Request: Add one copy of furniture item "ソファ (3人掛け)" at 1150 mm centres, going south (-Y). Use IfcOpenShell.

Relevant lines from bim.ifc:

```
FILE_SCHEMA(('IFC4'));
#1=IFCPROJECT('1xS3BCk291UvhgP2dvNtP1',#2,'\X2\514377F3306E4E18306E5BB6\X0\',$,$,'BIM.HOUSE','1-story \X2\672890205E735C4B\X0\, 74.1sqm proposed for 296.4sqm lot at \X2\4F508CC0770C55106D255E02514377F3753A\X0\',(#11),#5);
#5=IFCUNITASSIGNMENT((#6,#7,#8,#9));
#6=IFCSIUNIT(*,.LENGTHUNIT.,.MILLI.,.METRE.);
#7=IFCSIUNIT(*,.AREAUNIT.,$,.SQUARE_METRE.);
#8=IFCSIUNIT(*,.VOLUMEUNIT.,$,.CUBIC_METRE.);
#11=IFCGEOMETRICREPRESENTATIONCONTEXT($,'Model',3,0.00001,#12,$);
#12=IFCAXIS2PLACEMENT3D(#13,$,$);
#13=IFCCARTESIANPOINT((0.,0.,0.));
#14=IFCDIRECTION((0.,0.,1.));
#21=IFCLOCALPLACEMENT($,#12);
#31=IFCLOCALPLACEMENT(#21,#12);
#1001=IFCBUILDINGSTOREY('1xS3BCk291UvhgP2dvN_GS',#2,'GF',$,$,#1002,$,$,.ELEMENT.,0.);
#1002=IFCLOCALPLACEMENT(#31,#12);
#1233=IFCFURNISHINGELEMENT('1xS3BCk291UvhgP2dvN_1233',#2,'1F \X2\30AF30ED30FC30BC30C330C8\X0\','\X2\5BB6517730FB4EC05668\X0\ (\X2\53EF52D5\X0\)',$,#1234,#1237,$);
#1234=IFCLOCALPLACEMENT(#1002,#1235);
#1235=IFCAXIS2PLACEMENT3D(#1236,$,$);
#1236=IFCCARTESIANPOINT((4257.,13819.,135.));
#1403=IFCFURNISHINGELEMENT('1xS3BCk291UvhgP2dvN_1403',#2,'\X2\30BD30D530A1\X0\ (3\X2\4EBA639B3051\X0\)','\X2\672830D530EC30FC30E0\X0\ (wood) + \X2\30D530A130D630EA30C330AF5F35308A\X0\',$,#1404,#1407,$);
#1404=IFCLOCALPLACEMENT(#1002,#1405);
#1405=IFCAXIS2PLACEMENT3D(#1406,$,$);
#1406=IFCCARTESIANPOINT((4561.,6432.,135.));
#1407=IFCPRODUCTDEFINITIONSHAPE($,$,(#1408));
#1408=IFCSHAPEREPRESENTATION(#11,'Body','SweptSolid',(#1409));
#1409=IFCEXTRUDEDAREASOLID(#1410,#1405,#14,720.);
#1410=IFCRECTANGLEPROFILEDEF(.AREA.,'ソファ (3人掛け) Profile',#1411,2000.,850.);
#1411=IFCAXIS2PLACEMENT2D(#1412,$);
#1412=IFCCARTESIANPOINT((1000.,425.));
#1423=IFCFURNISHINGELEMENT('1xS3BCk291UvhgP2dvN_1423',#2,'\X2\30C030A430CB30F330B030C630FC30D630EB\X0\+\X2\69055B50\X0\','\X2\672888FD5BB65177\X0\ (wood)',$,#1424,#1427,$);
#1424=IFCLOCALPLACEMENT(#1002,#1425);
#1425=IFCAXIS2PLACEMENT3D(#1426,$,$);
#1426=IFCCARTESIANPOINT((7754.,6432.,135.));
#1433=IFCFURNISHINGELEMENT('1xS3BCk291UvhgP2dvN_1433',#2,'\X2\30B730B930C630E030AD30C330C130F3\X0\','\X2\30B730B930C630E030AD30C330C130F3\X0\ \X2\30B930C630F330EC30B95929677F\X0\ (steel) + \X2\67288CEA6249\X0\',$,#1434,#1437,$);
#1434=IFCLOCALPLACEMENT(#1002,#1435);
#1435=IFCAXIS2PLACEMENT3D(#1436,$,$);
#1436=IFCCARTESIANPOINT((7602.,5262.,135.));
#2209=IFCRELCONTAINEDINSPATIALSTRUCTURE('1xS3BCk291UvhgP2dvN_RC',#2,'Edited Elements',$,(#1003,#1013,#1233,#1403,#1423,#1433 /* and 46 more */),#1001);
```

```python
import numpy as np
import ifcopenshell
import ifcopenshell.api.geometry
import ifcopenshell.api.root
import ifcopenshell.util.element
import ifcopenshell.util.placement

model = ifcopenshell.open("bim.ifc")


def reuse_history(source, copy):
    """copy_class also copies each property set's owner history, people and application; keep the originals."""
    for rel in copy.IsDefinedBy:
        if rel.is_a("IfcRelDefinesByProperties") and (history := rel.RelatingPropertyDefinition.OwnerHistory):
            rel.RelatingPropertyDefinition.OwnerHistory = source.OwnerHistory
            ifcopenshell.util.element.remove_deep2(model, history)


source = model.by_id(1403)
base = ifcopenshell.util.placement.get_local_placement(source.ObjectPlacement)
step = np.array([0.0, -1.0, 0.0]) * 1150.0

for i in range(1, 2):
    copy = ifcopenshell.api.root.copy_class(model, product=source)
    copy.Representation = ifcopenshell.util.element.copy_deep(
        model, source.Representation, exclude=["IfcGeometricRepresentationContext", "IfcRepresentationMap"]
    )
    reuse_history(source, copy)
    matrix = base.copy()
    matrix[:3, 3] += i * step
    print("added at", matrix[:3, 3].round(3) + 0.0)
    ifcopenshell.api.geometry.edit_object_placement(model, product=copy, matrix=matrix, is_si=False)

model.write("bim_edited.ifc")
```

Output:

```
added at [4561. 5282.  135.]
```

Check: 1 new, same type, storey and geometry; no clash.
